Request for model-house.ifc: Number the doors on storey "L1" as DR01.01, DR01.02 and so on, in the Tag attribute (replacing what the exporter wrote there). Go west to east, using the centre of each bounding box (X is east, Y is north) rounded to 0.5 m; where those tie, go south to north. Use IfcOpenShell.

First a look at what the model holds.

```python
import ifcopenshell
import ifcopenshell.util.element
import ifcopenshell.util.placement

model = ifcopenshell.open("model-house.ifc")
print(model.schema)
storey = next(s for s in model.by_type("IfcBuildingStorey") if s.Name == "L1")
doors = [e for e in ifcopenshell.util.element.get_decomposition(storey) if e.is_a("IfcDoor")]
for e in sorted(doors, key=lambda e: e.id()):
    origin = ifcopenshell.util.placement.get_local_placement(e.ObjectPlacement)[:3, 3]
    print(e.id(), e.Tag, e.Name, origin.round(2) + 0.0, sep=" | ")
```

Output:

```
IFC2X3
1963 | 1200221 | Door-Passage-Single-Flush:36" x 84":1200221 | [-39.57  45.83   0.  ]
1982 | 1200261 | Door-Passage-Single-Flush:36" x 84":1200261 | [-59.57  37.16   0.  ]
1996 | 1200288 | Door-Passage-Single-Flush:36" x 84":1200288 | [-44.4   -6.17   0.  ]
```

```python
import ifcopenshell
import ifcopenshell.geom
import ifcopenshell.util.element
import ifcopenshell.util.shape

model = ifcopenshell.open("model-house.ifc")
settings = ifcopenshell.geom.settings()
settings.set("use-world-coords", True)


def centre(element):
    shape = ifcopenshell.geom.create_shape(settings, element)
    return ifcopenshell.util.shape.get_bbox_centroid(shape.geometry)


storey = next(s for s in model.by_type("IfcBuildingStorey") if s.Name == "L1")
doors = [e for e in ifcopenshell.util.element.get_decomposition(storey) if e.is_a("IfcDoor")]

# Insertion points can sit at a corner or the storey origin, so sort by the geometry (in metres).
centres = {e: centre(e) for e in doors}
doors.sort(key=lambda e: (round(centres[e][0] / 0.5), centres[e][1]))

for i, e in enumerate(doors, start=1):
    number = f"DR01.{i:02d}"
    e.Tag = number
    print(e.id(), number)

model.write("model-house_rev.ifc")
```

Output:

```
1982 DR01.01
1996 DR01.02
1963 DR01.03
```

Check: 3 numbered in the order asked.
